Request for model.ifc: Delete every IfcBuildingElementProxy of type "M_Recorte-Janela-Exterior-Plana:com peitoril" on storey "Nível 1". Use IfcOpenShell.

First a look at what the model holds.

```python
import ifcopenshell
import ifcopenshell.util.element

model = ifcopenshell.open("model.ifc")
print(model.schema)
storey = next(s for s in model.by_type("IfcBuildingStorey") if s.Name == "Nível 1")
proxies = [e for e in ifcopenshell.util.element.get_decomposition(storey) if e.is_a("IfcBuildingElementProxy")]
seen = {}
for e in proxies:
    element_type = ifcopenshell.util.element.get_type(e)
    name = element_type.Name if element_type not in (None, e) else None
    seen[name] = seen.get(name, 0) + 1
for name, count in sorted(seen.items(), key=str):
    print(count, "x", name)
```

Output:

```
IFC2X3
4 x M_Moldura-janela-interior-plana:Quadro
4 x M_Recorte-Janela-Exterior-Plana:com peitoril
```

```python
import ifcopenshell
import ifcopenshell.api.root
import ifcopenshell.util.element

model = ifcopenshell.open("model.ifc")

storey = next(s for s in model.by_type("IfcBuildingStorey") if s.Name == "Nível 1")
proxies = [e for e in ifcopenshell.util.element.get_decomposition(storey) if e.is_a("IfcBuildingElementProxy")]
targets = [e for e in proxies if (t := ifcopenshell.util.element.get_type(e)) not in (None, e) and t.Name == "M_Recorte-Janela-Exterior-Plana:com peitoril"]

for e in targets:
    ifcopenshell.api.root.remove_product(model, product=e)
print(len(targets), "removed")

model.write("model-out.ifc")
```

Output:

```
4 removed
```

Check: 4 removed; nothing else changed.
